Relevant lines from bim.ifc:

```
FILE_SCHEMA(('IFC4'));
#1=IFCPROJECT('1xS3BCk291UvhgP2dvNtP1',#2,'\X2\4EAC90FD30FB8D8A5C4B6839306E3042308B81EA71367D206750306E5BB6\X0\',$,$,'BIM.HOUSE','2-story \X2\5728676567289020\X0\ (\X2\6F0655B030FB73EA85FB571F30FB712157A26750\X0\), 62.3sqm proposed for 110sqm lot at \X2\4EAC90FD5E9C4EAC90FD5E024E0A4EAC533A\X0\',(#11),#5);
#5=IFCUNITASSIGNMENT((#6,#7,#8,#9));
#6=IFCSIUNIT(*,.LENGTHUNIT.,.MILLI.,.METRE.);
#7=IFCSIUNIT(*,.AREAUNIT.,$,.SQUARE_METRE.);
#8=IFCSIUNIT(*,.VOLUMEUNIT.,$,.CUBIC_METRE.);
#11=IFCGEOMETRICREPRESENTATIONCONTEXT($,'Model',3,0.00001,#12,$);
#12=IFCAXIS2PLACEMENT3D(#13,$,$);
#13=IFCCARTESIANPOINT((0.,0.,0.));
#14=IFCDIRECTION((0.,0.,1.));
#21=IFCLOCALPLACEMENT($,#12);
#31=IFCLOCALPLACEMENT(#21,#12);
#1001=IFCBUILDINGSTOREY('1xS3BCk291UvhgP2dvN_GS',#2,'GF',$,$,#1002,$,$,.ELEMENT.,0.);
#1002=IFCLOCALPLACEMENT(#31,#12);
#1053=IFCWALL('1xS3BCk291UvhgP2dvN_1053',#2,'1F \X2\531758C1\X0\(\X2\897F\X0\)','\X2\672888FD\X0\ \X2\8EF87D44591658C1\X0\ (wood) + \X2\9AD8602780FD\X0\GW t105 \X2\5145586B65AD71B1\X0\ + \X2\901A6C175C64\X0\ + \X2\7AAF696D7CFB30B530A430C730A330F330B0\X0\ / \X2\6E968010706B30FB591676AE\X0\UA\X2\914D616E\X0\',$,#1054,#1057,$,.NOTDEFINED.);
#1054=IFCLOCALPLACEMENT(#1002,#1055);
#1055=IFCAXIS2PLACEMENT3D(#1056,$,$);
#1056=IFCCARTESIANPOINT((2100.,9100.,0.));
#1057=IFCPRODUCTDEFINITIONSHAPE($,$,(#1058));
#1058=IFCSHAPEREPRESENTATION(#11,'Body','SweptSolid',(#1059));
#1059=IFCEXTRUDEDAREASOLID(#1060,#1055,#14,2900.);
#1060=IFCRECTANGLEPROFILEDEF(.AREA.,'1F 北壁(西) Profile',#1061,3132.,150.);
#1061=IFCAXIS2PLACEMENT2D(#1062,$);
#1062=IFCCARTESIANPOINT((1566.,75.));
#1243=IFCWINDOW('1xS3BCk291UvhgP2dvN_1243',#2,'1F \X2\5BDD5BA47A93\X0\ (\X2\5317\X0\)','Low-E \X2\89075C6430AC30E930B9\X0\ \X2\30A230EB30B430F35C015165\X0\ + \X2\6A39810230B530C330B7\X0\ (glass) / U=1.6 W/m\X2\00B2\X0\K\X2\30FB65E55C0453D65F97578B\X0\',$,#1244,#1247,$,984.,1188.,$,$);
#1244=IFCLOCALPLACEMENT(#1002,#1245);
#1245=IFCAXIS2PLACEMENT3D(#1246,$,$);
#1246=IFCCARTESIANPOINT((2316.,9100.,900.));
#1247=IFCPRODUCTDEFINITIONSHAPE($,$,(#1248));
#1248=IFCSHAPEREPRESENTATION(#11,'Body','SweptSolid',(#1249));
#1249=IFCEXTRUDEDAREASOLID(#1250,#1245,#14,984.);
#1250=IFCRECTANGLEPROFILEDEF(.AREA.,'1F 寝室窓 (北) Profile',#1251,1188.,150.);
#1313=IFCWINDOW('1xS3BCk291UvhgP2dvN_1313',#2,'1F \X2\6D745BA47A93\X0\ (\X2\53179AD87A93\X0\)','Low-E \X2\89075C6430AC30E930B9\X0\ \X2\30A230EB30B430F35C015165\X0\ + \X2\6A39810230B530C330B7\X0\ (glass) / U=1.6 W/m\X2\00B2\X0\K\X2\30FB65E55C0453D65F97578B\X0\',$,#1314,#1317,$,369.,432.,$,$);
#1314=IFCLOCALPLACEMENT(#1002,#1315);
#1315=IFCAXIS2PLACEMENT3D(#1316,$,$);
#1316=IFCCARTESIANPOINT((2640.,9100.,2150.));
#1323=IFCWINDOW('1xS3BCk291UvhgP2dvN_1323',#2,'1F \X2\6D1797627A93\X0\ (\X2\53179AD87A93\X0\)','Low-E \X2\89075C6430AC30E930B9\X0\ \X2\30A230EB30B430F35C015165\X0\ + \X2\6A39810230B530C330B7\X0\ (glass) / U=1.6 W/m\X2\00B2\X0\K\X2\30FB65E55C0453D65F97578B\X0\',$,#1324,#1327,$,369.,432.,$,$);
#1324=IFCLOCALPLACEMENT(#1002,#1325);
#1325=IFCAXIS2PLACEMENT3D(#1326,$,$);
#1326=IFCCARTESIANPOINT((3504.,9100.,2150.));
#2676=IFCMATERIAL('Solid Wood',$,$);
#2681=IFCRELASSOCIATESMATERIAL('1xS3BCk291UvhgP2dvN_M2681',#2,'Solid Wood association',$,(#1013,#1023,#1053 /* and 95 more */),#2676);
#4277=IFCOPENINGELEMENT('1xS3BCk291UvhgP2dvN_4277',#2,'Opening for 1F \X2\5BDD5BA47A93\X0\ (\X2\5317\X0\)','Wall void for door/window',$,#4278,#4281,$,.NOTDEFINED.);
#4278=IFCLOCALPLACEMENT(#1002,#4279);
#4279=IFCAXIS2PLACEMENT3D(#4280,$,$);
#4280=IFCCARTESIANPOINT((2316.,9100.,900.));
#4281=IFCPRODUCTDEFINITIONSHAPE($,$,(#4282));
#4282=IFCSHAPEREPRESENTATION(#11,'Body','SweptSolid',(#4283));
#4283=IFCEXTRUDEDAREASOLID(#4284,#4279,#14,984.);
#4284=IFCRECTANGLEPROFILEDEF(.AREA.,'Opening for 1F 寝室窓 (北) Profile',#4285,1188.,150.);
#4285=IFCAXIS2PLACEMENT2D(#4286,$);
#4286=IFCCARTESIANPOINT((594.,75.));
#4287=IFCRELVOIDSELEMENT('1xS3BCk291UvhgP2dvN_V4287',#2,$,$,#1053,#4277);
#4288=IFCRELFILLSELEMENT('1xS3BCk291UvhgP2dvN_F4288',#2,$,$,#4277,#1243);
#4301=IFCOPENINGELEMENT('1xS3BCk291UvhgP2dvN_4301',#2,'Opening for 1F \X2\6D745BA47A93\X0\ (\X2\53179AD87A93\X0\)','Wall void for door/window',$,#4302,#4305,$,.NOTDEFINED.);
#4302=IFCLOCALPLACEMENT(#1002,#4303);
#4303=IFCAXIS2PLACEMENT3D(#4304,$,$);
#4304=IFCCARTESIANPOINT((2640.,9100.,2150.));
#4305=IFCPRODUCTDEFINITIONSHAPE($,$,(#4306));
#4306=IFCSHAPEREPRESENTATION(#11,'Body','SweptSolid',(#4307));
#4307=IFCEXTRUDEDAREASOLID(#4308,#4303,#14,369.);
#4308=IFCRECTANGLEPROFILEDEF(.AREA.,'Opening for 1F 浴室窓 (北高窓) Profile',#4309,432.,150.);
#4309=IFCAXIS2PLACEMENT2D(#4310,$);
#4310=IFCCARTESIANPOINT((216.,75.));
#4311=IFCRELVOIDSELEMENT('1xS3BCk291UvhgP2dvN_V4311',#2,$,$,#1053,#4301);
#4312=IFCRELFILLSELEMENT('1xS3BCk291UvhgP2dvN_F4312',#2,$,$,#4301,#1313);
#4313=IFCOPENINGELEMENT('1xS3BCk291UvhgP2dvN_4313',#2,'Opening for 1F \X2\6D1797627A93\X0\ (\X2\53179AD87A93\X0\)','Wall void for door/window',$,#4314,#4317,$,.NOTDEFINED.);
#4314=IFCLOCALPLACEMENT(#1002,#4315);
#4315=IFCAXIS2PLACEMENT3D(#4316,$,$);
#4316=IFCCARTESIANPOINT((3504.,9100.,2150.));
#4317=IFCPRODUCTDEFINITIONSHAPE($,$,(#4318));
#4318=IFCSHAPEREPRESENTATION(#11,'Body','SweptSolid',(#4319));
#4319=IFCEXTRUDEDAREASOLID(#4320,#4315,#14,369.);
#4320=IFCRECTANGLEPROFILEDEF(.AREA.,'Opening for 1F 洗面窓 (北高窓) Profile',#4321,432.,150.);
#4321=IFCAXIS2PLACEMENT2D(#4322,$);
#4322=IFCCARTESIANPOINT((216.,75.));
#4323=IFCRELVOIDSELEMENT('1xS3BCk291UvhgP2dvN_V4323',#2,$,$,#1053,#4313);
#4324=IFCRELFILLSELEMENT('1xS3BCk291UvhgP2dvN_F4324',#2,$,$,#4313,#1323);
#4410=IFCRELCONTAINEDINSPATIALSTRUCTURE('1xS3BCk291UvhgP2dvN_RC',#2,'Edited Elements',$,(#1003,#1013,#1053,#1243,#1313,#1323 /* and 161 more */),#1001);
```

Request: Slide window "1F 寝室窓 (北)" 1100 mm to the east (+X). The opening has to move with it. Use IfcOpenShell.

```python
import ifcopenshell
import ifcopenshell.api.geometry
import ifcopenshell.util.placement
import ifcopenshell.util.unit

model = ifcopenshell.open("bim.ifc")
unit_scale = ifcopenshell.util.unit.calculate_unit_scale(model)

window = model.by_guid("1xS3BCk291UvhgP2dvN_1243")
opening = window.FillsVoids[0].RelatingOpeningElement
wall = opening.VoidsElements[0].RelatingBuildingElement

wall_matrix = ifcopenshell.util.placement.get_local_placement(wall.ObjectPlacement)
shift = wall_matrix[:3, 0] * 1.1 / unit_scale
before = ifcopenshell.util.placement.get_local_placement(window.ObjectPlacement)[:3, 3].copy()

# The window is not placed relative to its opening, so move both.
for product in (opening, window):
    matrix = ifcopenshell.util.placement.get_local_placement(product.ObjectPlacement)
    matrix[:3, 3] += shift
    ifcopenshell.api.geometry.edit_object_placement(model, product=product, matrix=matrix, is_si=False)

after = ifcopenshell.util.placement.get_local_placement(window.ObjectPlacement)[:3, 3]
print("window moved by", (after - before).round(3) + 0.0)

model.write("bim_v2.ifc")
```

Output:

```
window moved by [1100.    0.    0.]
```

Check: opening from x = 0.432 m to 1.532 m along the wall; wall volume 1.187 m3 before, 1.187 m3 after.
